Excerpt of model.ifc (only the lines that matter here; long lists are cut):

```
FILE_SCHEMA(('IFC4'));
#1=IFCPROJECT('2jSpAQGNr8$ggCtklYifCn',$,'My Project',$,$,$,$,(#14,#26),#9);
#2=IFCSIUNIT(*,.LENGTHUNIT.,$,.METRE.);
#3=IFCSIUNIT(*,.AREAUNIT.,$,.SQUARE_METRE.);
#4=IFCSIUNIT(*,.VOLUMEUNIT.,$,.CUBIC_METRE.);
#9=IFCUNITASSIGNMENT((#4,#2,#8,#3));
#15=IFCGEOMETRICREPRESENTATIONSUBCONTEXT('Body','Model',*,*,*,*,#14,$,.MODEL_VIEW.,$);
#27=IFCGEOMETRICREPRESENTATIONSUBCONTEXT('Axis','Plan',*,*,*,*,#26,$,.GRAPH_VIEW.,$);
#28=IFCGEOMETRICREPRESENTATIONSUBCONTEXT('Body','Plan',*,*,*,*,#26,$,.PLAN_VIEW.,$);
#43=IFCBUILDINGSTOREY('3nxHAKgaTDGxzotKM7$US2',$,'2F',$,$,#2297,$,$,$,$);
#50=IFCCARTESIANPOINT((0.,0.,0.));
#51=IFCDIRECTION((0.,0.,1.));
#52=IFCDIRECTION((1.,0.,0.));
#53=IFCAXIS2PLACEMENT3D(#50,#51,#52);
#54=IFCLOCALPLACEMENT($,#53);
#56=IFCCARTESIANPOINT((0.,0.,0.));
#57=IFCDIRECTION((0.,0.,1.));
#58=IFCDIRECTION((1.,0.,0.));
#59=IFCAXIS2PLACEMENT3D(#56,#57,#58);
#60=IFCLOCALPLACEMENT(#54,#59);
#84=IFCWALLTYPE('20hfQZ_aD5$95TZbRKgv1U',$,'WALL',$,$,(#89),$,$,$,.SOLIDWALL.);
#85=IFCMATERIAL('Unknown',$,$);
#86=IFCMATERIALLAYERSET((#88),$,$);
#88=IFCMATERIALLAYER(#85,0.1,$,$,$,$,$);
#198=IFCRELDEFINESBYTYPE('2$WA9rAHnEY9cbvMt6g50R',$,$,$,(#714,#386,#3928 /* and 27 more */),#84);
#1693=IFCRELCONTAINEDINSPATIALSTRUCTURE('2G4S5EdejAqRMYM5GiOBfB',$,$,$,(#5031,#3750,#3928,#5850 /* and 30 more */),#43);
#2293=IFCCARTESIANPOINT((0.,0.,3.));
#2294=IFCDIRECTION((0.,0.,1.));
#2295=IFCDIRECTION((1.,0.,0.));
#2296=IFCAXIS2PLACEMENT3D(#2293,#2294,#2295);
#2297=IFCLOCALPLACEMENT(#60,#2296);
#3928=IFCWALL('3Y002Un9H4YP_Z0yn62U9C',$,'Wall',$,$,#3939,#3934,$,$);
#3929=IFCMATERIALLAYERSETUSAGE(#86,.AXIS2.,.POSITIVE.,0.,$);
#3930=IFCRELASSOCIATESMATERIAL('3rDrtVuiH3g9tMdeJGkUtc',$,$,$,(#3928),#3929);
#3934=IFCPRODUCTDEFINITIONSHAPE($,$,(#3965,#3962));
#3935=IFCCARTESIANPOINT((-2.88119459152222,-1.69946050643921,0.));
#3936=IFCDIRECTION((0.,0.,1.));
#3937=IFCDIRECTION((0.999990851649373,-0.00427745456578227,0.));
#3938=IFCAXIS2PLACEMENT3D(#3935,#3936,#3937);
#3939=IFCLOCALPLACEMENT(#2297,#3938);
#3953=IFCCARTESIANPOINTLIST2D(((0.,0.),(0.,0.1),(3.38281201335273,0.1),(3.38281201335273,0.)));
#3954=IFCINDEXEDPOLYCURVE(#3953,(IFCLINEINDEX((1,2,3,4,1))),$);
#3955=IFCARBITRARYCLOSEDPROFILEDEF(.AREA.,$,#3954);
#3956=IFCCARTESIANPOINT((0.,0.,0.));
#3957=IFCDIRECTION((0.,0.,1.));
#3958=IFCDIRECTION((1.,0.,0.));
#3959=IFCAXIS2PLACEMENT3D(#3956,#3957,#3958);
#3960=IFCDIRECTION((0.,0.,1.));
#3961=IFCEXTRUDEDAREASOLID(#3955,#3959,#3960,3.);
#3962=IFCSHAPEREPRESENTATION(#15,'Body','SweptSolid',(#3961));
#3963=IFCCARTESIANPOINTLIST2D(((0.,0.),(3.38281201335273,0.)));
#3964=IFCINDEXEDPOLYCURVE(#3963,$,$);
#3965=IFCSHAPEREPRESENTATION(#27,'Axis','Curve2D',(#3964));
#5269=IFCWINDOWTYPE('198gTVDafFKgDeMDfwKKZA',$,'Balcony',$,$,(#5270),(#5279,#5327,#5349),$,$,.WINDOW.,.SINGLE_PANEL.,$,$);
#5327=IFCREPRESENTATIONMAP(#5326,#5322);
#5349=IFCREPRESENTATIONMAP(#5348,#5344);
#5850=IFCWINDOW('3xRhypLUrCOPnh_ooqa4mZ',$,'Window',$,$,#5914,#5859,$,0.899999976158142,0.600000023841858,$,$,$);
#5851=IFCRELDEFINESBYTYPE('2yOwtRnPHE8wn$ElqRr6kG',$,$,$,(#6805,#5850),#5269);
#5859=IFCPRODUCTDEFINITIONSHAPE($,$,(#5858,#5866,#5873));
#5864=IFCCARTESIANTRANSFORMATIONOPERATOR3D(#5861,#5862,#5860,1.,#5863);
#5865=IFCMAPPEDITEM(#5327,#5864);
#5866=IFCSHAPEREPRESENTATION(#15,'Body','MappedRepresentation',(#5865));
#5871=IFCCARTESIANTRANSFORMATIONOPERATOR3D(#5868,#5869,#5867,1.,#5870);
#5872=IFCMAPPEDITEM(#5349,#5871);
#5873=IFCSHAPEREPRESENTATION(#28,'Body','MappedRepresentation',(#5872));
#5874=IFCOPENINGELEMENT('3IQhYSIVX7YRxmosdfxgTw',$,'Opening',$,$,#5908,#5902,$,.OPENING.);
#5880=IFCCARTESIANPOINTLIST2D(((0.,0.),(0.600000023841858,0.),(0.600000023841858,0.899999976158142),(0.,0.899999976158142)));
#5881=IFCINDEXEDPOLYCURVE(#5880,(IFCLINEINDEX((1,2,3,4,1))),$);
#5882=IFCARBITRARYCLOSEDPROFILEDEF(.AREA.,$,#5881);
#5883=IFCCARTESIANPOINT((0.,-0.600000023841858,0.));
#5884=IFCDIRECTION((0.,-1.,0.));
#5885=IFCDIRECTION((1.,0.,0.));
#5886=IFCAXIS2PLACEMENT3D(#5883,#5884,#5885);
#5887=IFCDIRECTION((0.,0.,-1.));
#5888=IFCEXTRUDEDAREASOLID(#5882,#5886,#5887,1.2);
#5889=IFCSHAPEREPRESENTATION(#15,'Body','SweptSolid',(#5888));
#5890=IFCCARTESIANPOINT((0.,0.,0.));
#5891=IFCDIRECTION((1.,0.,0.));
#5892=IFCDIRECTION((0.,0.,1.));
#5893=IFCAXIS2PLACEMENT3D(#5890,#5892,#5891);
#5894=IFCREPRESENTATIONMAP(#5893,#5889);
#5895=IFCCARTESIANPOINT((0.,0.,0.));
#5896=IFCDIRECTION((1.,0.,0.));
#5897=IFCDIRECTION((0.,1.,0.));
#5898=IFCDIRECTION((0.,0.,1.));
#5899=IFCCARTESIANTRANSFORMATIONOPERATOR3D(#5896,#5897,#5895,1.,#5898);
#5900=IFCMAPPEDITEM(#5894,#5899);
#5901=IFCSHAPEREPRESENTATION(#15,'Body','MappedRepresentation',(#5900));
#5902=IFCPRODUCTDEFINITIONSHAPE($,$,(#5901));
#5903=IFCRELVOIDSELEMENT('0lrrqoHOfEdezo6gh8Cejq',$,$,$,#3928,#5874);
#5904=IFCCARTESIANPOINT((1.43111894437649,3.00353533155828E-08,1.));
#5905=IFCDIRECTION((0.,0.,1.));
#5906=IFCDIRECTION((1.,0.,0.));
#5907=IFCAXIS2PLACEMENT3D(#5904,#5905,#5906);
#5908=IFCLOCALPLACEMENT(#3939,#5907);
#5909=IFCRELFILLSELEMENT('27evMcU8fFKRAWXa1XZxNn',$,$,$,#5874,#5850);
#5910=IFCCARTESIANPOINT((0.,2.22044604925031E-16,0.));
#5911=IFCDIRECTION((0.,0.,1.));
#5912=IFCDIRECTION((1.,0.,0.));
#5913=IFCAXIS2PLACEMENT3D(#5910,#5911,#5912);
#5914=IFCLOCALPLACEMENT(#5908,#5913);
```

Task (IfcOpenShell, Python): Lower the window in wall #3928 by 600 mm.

```python
import numpy as np
import ifcopenshell
import ifcopenshell.api.geometry
import ifcopenshell.util.placement
import ifcopenshell.util.unit

model = ifcopenshell.open("model.ifc")
unit_scale = ifcopenshell.util.unit.calculate_unit_scale(model)

window = model.by_guid("3xRhypLUrCOPnh_ooqa4mZ")
opening = window.FillsVoids[0].RelatingOpeningElement
dz = -0.6 / unit_scale

shift = np.array([0.0, 0.0, dz])
# The window is placed relative to its opening, so it follows when the opening moves.
matrix = ifcopenshell.util.placement.get_local_placement(opening.ObjectPlacement)
matrix[:3, 3] += shift
ifcopenshell.api.geometry.edit_object_placement(
    model, product=opening, matrix=matrix, is_si=False, should_transform_children=True
)

print(f"moved by {dz * unit_scale:+.3f} m")

model.write("model_rev.ifc")
```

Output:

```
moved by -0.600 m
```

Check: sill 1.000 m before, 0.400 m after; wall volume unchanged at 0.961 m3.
